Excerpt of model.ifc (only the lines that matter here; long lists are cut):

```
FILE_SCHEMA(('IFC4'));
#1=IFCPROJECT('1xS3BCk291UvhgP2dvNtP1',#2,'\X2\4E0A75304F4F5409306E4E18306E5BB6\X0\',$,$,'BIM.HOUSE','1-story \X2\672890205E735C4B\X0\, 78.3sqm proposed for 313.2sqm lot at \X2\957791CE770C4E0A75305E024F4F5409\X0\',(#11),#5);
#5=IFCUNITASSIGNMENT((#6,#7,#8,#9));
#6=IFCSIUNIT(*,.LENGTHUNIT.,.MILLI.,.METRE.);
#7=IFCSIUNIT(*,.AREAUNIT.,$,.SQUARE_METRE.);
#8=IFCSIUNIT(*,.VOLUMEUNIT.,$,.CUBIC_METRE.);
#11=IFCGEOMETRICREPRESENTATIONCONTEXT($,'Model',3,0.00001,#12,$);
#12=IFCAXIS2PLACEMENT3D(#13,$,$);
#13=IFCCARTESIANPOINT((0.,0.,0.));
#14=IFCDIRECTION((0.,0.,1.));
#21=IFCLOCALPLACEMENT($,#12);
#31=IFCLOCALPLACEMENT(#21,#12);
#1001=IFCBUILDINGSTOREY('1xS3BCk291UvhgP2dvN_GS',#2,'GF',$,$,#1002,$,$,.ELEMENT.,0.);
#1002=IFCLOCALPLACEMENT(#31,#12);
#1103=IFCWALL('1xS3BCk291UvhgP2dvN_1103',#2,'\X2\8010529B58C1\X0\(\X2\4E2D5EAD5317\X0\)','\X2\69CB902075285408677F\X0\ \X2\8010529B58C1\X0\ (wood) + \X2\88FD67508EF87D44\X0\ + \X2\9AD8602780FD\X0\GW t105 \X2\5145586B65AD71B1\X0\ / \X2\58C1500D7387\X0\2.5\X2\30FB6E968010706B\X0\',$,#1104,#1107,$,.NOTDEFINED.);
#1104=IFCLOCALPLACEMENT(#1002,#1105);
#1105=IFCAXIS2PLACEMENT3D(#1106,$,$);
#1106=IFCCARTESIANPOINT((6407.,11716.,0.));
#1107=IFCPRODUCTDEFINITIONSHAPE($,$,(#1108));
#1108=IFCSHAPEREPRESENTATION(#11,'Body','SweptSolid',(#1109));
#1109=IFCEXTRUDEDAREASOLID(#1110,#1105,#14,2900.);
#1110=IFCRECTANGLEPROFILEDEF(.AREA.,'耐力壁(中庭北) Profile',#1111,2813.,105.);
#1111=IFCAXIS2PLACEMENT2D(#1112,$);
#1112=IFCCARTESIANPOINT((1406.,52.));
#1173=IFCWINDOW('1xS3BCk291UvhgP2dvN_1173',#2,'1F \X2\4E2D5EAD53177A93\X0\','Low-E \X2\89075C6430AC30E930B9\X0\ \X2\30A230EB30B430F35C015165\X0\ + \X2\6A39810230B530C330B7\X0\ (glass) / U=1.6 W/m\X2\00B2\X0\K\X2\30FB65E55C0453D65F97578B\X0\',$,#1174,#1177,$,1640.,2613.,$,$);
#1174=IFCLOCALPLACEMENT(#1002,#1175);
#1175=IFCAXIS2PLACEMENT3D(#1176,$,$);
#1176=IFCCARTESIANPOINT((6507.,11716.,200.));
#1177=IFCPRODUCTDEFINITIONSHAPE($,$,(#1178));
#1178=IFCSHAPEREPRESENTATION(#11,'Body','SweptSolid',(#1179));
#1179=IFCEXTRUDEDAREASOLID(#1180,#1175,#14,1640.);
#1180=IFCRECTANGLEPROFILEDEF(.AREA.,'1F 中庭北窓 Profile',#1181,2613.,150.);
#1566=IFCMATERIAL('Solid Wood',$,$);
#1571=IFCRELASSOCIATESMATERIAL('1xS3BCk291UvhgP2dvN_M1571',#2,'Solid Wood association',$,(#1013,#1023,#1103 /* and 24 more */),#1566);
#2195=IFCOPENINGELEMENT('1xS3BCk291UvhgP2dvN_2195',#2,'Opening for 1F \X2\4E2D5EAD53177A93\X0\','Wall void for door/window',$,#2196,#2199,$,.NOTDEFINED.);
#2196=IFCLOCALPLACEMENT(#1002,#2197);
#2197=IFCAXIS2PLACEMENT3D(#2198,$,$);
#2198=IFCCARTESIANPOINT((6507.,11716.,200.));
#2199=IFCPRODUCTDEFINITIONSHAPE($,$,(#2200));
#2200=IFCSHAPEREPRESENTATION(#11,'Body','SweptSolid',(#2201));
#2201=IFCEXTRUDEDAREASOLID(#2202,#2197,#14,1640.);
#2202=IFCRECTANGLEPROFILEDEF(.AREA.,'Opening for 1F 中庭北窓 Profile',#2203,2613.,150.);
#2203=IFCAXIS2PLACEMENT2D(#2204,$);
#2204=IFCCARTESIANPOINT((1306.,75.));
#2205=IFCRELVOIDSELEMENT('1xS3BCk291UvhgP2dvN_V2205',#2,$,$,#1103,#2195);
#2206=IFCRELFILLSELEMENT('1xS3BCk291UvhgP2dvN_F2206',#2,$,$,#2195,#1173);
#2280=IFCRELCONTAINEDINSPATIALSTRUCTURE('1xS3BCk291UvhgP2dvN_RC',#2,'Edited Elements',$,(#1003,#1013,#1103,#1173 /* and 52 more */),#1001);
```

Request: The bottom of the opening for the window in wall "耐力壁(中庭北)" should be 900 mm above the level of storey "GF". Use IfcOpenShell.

```python
import numpy as np
import ifcopenshell
import ifcopenshell.api.geometry
import ifcopenshell.geom
import ifcopenshell.util.element
import ifcopenshell.util.placement
import ifcopenshell.util.shape
import ifcopenshell.util.unit

model = ifcopenshell.open("model.ifc")
unit_scale = ifcopenshell.util.unit.calculate_unit_scale(model)

window = model.by_guid("1xS3BCk291UvhgP2dvN_1173")
opening = window.FillsVoids[0].RelatingOpeningElement
storey = ifcopenshell.util.element.get_container(window, ifc_class="IfcBuildingStorey")
level = ifcopenshell.util.placement.get_local_placement(storey.ObjectPlacement)[2, 3]

# The opening's origin need not be at the sill, so measure its lowest point.
shape = ifcopenshell.geom.create_shape(ifcopenshell.geom.settings(), opening)
bottom = ifcopenshell.util.shape.get_shape_bottom_elevation(shape, shape.geometry) / unit_scale
dz = level + 900.0 - bottom

shift = np.array([0.0, 0.0, dz])
# The window is not placed relative to its opening, so move both.
for product in (opening, window):
    matrix = ifcopenshell.util.placement.get_local_placement(product.ObjectPlacement)
    matrix[:3, 3] += shift
    ifcopenshell.api.geometry.edit_object_placement(model, product=product, matrix=matrix, is_si=False)

print(f"moved by {dz * unit_scale:+.3f} m")

model.write("model_v2.ifc")
```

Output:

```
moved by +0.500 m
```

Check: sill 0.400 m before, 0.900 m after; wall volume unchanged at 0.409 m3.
